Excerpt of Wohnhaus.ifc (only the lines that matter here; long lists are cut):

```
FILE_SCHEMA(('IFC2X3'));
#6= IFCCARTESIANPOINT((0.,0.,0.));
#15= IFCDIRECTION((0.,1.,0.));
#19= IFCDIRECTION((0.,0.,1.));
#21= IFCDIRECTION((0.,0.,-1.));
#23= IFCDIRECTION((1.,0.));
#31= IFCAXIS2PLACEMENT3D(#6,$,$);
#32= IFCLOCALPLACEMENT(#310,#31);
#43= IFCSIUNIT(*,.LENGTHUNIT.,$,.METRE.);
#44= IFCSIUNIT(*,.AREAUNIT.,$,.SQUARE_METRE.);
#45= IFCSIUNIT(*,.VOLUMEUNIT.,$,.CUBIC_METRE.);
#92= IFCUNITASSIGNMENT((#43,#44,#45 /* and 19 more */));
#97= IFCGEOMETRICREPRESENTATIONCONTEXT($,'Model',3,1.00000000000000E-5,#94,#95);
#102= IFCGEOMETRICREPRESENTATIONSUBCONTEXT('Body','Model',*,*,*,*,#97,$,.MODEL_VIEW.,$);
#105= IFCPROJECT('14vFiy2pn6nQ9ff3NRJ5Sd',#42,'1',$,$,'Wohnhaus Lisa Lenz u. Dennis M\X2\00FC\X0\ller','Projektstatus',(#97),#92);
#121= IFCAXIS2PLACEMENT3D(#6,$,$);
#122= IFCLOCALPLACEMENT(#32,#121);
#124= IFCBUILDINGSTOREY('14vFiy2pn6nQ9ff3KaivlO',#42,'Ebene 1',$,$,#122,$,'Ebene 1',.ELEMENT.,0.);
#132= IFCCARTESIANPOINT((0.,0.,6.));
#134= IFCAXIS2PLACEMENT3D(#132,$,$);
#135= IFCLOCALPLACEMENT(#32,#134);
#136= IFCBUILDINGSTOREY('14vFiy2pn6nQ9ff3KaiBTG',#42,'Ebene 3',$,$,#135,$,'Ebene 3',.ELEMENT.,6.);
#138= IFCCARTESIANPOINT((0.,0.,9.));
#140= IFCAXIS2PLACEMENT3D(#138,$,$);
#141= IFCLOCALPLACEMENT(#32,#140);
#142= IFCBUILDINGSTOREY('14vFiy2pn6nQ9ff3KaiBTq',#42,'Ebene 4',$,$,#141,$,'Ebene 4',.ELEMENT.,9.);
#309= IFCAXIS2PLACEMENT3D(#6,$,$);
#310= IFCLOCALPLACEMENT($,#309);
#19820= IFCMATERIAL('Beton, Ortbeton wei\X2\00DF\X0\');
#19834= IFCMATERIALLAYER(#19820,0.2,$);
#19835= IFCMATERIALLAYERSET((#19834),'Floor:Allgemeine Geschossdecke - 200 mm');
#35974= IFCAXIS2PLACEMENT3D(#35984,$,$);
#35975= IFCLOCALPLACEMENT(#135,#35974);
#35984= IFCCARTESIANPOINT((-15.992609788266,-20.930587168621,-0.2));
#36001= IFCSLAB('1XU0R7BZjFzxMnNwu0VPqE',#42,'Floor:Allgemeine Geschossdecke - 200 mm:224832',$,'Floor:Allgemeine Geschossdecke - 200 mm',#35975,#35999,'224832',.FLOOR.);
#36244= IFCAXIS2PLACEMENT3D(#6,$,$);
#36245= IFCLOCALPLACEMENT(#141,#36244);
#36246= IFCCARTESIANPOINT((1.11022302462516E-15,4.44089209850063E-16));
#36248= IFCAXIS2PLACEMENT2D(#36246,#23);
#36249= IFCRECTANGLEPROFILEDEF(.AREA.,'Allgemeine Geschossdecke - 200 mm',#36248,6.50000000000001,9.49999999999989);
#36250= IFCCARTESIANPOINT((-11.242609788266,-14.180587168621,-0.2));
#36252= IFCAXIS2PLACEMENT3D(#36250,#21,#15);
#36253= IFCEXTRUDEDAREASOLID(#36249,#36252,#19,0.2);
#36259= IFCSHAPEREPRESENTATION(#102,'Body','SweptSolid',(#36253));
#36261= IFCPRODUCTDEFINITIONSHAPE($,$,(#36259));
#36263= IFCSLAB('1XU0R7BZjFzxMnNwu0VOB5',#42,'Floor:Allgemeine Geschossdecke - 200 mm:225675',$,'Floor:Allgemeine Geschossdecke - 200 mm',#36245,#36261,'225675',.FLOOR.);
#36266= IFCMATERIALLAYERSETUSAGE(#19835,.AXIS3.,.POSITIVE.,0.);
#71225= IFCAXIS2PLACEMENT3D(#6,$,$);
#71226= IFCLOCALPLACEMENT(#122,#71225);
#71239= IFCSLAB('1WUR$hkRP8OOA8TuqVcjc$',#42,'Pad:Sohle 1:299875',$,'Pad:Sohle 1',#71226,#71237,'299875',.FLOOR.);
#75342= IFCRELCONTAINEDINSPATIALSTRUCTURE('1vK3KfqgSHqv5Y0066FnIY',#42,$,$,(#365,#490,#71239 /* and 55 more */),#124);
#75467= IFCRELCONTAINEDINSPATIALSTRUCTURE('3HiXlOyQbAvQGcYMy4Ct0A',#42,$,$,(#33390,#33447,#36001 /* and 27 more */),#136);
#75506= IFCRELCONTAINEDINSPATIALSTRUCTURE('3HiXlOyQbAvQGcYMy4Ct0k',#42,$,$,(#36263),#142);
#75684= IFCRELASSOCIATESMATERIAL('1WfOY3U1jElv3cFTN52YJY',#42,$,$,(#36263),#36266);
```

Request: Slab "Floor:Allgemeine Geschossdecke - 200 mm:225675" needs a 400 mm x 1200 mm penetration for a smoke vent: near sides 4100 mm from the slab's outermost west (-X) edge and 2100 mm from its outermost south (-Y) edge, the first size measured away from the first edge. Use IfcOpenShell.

```python
import numpy as np
import ifcopenshell
import ifcopenshell.api.feature
import ifcopenshell.api.geometry
import ifcopenshell.api.root
import ifcopenshell.geom
import ifcopenshell.util.placement
import ifcopenshell.util.representation
import ifcopenshell.util.shape
import ifcopenshell.util.unit

model = ifcopenshell.open("Wohnhaus.ifc")
unit_scale = ifcopenshell.util.unit.calculate_unit_scale(model)
settings = ifcopenshell.geom.settings()


def volume(element):
    """Net volume in cubic metres, openings subtracted."""
    shape = ifcopenshell.geom.create_shape(settings, element)
    return ifcopenshell.util.shape.get_volume(shape.geometry)


slab = model.by_guid("1XU0R7BZjFzxMnNwu0VOB5")
before = volume(slab)

# Extent in the slab's own axes, in metres. The edges named are its -X and -Y sides.
slab_shape = ifcopenshell.geom.create_shape(settings, slab)
vertices = ifcopenshell.util.shape.get_vertices(slab_shape.geometry)
x_min, y_min, bottom = vertices.min(axis=0)
top = vertices[:, 2].max()

opening = ifcopenshell.api.root.create_entity(model, ifc_class="IfcOpeningElement", name="Smoke vent opening")
context = ifcopenshell.util.representation.get_context(model, "Model", "Body", "MODEL_VIEW")
width, depth = 0.4, 1.2
outline = [(0.0, 0.0), (width, 0.0), (width, depth), (0.0, depth), (0.0, 0.0)]
# Overshoot both faces by 50 mm so the cut is clean.
shape = ifcopenshell.api.geometry.add_slab_representation(
    model, context=context, depth=top - bottom + 0.1, polyline=outline
)
ifcopenshell.api.geometry.assign_representation(model, product=opening, representation=shape)

matrix = ifcopenshell.util.placement.get_local_placement(slab.ObjectPlacement)
matrix[:, 3] = matrix @ np.append(np.array([x_min + 4.1, y_min + 2.1, bottom - 0.05]) / unit_scale, 1.0)
ifcopenshell.api.geometry.edit_object_placement(model, product=opening, matrix=matrix, is_si=False)
ifcopenshell.api.feature.add_feature(model, feature=opening, element=slab)

after = volume(slab)

print(f"slab volume {before:.3f} -> {after:.3f} m3")

model.write("Wohnhaus_edited.ifc")
```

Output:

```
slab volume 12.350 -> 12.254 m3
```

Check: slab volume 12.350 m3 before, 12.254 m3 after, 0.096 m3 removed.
